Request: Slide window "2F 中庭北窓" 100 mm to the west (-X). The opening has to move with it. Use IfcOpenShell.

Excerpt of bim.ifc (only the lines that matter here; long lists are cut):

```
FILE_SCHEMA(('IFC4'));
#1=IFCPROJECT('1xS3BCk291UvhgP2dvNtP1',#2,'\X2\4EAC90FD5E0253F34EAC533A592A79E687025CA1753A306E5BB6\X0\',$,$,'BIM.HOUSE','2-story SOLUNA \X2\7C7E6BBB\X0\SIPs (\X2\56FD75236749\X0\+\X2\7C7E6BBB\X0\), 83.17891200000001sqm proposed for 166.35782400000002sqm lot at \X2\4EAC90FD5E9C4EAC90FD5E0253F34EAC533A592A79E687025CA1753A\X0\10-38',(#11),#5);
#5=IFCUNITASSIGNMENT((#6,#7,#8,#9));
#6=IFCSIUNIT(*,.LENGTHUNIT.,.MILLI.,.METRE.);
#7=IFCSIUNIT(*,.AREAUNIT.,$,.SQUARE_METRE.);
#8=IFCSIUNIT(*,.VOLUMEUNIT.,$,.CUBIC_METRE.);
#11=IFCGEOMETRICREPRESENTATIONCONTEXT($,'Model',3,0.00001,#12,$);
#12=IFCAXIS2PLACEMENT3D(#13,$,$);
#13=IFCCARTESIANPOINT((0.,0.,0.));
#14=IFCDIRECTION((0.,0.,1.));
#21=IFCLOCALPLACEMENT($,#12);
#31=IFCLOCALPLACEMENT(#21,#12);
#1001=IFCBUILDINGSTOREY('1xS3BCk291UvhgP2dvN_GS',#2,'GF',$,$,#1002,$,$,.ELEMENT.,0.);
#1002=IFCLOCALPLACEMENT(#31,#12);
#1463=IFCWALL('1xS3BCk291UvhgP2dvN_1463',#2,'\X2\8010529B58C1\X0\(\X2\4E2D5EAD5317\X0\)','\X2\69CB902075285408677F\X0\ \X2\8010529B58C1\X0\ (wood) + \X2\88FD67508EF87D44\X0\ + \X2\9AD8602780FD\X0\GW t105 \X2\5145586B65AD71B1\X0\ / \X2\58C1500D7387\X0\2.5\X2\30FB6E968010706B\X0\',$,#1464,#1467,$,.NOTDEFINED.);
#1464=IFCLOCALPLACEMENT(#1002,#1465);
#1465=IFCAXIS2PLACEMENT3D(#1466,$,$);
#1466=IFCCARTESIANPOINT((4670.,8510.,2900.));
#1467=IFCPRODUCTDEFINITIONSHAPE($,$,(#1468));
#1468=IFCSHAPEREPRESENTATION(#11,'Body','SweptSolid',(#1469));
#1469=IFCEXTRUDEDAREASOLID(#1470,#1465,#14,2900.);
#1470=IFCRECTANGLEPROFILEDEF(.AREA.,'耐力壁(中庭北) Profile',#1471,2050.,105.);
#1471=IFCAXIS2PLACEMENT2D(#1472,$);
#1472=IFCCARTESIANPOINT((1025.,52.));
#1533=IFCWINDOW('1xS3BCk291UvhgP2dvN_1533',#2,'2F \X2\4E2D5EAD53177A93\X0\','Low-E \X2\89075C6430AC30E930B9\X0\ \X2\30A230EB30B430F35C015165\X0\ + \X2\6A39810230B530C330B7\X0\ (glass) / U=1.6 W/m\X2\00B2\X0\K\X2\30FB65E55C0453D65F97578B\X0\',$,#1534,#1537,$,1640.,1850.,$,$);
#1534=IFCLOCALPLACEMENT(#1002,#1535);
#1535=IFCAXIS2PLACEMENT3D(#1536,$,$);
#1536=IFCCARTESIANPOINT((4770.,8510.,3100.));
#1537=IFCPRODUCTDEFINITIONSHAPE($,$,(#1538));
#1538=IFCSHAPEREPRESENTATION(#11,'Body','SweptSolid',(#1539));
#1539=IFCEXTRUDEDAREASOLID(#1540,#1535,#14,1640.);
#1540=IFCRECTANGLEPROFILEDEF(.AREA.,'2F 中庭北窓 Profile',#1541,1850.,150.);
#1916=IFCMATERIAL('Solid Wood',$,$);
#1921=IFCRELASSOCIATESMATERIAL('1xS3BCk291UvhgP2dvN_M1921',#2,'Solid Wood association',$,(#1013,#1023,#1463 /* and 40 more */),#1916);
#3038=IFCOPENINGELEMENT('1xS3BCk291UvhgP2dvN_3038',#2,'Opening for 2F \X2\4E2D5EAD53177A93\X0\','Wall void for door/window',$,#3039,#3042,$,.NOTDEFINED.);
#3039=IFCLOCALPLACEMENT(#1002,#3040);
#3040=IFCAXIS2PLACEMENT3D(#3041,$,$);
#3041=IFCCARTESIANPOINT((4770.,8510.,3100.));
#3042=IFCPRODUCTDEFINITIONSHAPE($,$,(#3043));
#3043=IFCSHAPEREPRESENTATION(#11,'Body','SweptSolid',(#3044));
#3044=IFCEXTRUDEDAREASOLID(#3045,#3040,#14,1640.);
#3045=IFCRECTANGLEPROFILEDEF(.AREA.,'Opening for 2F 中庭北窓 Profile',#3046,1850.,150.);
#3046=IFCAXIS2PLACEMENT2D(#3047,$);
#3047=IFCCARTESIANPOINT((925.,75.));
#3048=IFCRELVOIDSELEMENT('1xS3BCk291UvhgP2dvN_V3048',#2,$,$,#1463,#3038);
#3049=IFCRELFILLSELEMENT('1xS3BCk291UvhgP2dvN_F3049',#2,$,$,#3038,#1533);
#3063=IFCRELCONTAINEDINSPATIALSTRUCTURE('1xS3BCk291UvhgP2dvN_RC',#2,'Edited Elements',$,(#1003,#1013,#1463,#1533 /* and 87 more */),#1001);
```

```python
import ifcopenshell
import ifcopenshell.api.geometry
import ifcopenshell.util.placement

model = ifcopenshell.open("bim.ifc")

window = model.by_id(1533)
opening = window.FillsVoids[0].RelatingOpeningElement
wall = opening.VoidsElements[0].RelatingBuildingElement

wall_matrix = ifcopenshell.util.placement.get_local_placement(wall.ObjectPlacement)
shift = wall_matrix[:3, 0] * -100.0
before = ifcopenshell.util.placement.get_local_placement(window.ObjectPlacement)[:3, 3].copy()

# The window is not placed relative to its opening, so move both.
for product in (opening, window):
    matrix = ifcopenshell.util.placement.get_local_placement(product.ObjectPlacement)
    matrix[:3, 3] += shift
    ifcopenshell.api.geometry.edit_object_placement(model, product=product, matrix=matrix, is_si=False)

after = ifcopenshell.util.placement.get_local_placement(window.ObjectPlacement)[:3, 3]
print("window moved by", (after - before).round(3) + 0.0)

model.write("bim_updated.ifc")
```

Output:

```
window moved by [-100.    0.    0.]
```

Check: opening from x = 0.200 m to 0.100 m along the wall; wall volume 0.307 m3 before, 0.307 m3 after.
